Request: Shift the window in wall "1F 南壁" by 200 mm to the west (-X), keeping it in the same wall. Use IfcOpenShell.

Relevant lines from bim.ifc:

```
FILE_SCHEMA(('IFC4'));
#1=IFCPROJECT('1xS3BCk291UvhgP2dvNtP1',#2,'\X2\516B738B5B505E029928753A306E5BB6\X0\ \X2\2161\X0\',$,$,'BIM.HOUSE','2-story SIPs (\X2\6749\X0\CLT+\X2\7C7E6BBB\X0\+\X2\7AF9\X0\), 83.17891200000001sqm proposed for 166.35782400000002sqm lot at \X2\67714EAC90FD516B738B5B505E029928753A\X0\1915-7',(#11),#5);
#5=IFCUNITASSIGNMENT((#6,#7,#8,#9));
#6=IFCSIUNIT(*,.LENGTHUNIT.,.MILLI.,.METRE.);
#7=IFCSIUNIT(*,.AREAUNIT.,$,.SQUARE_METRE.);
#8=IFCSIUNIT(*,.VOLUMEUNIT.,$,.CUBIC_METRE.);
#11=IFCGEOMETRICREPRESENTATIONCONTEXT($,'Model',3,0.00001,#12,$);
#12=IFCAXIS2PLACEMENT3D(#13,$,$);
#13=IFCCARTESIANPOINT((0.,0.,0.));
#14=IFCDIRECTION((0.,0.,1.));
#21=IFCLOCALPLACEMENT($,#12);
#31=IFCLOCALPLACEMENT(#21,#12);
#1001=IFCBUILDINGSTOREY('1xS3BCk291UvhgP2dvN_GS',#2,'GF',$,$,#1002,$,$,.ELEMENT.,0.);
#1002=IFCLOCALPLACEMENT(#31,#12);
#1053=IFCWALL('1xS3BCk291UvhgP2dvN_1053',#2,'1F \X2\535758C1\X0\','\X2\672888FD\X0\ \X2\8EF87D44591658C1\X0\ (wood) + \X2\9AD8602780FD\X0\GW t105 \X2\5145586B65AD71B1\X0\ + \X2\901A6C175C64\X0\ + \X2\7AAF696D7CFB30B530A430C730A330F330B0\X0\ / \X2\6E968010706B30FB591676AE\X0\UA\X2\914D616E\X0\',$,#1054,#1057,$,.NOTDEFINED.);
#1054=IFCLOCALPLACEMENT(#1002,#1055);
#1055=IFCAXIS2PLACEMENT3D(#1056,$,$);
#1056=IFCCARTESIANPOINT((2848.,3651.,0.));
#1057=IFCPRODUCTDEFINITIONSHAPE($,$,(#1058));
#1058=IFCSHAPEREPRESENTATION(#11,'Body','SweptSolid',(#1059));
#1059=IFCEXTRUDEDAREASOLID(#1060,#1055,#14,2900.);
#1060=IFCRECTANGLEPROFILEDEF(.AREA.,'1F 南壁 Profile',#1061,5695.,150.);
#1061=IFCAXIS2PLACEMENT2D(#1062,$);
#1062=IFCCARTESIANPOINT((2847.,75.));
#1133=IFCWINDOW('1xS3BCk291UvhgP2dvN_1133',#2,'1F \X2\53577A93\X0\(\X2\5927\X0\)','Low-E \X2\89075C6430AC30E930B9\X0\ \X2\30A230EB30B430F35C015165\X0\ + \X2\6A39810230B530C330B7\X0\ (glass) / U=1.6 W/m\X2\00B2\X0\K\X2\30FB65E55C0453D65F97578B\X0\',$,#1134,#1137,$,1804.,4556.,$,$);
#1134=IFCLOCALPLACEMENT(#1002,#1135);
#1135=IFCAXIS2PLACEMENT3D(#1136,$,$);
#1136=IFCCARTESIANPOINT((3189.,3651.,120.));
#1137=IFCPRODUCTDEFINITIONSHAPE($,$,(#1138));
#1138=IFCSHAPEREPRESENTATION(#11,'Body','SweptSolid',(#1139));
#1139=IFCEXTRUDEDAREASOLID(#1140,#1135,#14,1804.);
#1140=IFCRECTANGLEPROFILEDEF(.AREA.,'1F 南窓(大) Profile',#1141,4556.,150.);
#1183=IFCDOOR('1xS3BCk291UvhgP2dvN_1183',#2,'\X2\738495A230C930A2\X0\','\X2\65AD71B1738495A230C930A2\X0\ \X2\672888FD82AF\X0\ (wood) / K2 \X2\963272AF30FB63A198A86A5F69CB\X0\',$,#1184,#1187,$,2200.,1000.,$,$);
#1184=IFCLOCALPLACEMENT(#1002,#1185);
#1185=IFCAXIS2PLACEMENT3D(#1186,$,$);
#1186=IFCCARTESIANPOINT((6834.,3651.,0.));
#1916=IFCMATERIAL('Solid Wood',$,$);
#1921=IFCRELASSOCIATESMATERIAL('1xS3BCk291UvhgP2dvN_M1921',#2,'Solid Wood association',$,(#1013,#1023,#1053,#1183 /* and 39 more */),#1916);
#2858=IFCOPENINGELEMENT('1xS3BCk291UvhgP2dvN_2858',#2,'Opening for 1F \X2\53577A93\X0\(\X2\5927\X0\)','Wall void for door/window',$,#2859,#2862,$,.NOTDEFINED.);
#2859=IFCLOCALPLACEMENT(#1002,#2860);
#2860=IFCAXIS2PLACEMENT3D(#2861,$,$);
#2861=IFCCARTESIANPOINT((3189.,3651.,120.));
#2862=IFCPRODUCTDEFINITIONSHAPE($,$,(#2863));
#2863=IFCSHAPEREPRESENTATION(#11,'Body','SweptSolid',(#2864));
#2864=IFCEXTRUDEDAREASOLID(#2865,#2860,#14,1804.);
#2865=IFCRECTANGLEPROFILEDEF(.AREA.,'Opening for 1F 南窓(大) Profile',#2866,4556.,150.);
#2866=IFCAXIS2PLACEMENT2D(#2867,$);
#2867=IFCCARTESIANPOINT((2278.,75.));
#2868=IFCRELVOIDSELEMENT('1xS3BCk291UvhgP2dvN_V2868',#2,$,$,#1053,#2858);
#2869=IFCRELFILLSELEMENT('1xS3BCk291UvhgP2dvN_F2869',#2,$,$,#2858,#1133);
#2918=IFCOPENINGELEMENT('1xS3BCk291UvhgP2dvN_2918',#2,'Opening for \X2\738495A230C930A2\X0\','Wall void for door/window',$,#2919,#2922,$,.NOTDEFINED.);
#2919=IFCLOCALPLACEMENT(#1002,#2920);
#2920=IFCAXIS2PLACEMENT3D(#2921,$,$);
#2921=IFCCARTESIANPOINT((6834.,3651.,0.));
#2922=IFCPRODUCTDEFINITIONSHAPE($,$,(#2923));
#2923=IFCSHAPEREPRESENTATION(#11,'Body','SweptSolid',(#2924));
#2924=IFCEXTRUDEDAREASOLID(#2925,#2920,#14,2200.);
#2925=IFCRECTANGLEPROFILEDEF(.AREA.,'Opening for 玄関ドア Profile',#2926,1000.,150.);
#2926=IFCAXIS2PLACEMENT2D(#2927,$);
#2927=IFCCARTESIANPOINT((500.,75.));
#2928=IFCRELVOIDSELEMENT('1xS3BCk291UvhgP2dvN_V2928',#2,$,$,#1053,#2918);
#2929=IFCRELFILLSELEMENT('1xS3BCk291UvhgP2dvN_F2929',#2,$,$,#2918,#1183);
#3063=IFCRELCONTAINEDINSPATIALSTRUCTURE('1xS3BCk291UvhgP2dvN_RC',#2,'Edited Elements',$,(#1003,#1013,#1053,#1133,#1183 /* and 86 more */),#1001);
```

```python
import ifcopenshell
import ifcopenshell.api.geometry
import ifcopenshell.util.placement

model = ifcopenshell.open("bim.ifc")

window = model.by_id(1133)
opening = window.FillsVoids[0].RelatingOpeningElement
wall = opening.VoidsElements[0].RelatingBuildingElement

wall_matrix = ifcopenshell.util.placement.get_local_placement(wall.ObjectPlacement)
shift = wall_matrix[:3, 0] * -200.0
before = ifcopenshell.util.placement.get_local_placement(window.ObjectPlacement)[:3, 3].copy()

# The window is not placed relative to its opening, so move both.
for product in (opening, window):
    matrix = ifcopenshell.util.placement.get_local_placement(product.ObjectPlacement)
    matrix[:3, 3] += shift
    ifcopenshell.api.geometry.edit_object_placement(model, product=product, matrix=matrix, is_si=False)

after = ifcopenshell.util.placement.get_local_placement(window.ObjectPlacement)[:3, 3]
print("window moved by", (after - before).round(3) + 0.0)

model.write("bim-out.ifc")
```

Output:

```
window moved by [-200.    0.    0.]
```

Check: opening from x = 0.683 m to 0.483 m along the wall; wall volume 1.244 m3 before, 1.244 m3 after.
